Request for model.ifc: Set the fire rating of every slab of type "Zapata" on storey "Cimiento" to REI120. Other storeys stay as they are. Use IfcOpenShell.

First a look at what the model holds.

```python
import ifcopenshell
import ifcopenshell.util.element

model = ifcopenshell.open("model.ifc")
print(model.schema)
storey = next(s for s in model.by_type("IfcBuildingStorey") if s.Name == "Cimiento")
slabs = [e for e in ifcopenshell.util.element.get_decomposition(storey) if e.is_a("IfcSlab")]
seen = {}
for e in slabs:
    element_type = ifcopenshell.util.element.get_type(e)
    key = (element_type.Name if element_type != e and element_type else None, ifcopenshell.util.element.get_pset(e, "Pset_SlabCommon", "FireRating"))
    seen[key] = seen.get(key, 0) + 1
for (name, value), count in sorted(seen.items(), key=str):
    print(count, "x", name, "|", value)
```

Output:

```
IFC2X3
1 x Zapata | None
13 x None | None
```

```python
import ifcopenshell
import ifcopenshell.api.pset
import ifcopenshell.util.element

model = ifcopenshell.open("model.ifc")

storey = next(s for s in model.by_type("IfcBuildingStorey") if s.Name == "Cimiento")
slabs = [e for e in ifcopenshell.util.element.get_decomposition(storey) if e.is_a("IfcSlab")]

count = 0
for e in slabs:
    element_type = ifcopenshell.util.element.get_type(e)
    if element_type in (None, e) or element_type.Name != "Zapata":
        continue
    # add_pset returns the element's existing set when there is one.
    pset = ifcopenshell.api.pset.add_pset(model, product=e, name="Pset_SlabCommon")
    ifcopenshell.api.pset.edit_pset(model, pset=pset, properties={"FireRating": "REI120"})
    count += 1

print(count, "slabs updated")

model.write("model_rev.ifc")
```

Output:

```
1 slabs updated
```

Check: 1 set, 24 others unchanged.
